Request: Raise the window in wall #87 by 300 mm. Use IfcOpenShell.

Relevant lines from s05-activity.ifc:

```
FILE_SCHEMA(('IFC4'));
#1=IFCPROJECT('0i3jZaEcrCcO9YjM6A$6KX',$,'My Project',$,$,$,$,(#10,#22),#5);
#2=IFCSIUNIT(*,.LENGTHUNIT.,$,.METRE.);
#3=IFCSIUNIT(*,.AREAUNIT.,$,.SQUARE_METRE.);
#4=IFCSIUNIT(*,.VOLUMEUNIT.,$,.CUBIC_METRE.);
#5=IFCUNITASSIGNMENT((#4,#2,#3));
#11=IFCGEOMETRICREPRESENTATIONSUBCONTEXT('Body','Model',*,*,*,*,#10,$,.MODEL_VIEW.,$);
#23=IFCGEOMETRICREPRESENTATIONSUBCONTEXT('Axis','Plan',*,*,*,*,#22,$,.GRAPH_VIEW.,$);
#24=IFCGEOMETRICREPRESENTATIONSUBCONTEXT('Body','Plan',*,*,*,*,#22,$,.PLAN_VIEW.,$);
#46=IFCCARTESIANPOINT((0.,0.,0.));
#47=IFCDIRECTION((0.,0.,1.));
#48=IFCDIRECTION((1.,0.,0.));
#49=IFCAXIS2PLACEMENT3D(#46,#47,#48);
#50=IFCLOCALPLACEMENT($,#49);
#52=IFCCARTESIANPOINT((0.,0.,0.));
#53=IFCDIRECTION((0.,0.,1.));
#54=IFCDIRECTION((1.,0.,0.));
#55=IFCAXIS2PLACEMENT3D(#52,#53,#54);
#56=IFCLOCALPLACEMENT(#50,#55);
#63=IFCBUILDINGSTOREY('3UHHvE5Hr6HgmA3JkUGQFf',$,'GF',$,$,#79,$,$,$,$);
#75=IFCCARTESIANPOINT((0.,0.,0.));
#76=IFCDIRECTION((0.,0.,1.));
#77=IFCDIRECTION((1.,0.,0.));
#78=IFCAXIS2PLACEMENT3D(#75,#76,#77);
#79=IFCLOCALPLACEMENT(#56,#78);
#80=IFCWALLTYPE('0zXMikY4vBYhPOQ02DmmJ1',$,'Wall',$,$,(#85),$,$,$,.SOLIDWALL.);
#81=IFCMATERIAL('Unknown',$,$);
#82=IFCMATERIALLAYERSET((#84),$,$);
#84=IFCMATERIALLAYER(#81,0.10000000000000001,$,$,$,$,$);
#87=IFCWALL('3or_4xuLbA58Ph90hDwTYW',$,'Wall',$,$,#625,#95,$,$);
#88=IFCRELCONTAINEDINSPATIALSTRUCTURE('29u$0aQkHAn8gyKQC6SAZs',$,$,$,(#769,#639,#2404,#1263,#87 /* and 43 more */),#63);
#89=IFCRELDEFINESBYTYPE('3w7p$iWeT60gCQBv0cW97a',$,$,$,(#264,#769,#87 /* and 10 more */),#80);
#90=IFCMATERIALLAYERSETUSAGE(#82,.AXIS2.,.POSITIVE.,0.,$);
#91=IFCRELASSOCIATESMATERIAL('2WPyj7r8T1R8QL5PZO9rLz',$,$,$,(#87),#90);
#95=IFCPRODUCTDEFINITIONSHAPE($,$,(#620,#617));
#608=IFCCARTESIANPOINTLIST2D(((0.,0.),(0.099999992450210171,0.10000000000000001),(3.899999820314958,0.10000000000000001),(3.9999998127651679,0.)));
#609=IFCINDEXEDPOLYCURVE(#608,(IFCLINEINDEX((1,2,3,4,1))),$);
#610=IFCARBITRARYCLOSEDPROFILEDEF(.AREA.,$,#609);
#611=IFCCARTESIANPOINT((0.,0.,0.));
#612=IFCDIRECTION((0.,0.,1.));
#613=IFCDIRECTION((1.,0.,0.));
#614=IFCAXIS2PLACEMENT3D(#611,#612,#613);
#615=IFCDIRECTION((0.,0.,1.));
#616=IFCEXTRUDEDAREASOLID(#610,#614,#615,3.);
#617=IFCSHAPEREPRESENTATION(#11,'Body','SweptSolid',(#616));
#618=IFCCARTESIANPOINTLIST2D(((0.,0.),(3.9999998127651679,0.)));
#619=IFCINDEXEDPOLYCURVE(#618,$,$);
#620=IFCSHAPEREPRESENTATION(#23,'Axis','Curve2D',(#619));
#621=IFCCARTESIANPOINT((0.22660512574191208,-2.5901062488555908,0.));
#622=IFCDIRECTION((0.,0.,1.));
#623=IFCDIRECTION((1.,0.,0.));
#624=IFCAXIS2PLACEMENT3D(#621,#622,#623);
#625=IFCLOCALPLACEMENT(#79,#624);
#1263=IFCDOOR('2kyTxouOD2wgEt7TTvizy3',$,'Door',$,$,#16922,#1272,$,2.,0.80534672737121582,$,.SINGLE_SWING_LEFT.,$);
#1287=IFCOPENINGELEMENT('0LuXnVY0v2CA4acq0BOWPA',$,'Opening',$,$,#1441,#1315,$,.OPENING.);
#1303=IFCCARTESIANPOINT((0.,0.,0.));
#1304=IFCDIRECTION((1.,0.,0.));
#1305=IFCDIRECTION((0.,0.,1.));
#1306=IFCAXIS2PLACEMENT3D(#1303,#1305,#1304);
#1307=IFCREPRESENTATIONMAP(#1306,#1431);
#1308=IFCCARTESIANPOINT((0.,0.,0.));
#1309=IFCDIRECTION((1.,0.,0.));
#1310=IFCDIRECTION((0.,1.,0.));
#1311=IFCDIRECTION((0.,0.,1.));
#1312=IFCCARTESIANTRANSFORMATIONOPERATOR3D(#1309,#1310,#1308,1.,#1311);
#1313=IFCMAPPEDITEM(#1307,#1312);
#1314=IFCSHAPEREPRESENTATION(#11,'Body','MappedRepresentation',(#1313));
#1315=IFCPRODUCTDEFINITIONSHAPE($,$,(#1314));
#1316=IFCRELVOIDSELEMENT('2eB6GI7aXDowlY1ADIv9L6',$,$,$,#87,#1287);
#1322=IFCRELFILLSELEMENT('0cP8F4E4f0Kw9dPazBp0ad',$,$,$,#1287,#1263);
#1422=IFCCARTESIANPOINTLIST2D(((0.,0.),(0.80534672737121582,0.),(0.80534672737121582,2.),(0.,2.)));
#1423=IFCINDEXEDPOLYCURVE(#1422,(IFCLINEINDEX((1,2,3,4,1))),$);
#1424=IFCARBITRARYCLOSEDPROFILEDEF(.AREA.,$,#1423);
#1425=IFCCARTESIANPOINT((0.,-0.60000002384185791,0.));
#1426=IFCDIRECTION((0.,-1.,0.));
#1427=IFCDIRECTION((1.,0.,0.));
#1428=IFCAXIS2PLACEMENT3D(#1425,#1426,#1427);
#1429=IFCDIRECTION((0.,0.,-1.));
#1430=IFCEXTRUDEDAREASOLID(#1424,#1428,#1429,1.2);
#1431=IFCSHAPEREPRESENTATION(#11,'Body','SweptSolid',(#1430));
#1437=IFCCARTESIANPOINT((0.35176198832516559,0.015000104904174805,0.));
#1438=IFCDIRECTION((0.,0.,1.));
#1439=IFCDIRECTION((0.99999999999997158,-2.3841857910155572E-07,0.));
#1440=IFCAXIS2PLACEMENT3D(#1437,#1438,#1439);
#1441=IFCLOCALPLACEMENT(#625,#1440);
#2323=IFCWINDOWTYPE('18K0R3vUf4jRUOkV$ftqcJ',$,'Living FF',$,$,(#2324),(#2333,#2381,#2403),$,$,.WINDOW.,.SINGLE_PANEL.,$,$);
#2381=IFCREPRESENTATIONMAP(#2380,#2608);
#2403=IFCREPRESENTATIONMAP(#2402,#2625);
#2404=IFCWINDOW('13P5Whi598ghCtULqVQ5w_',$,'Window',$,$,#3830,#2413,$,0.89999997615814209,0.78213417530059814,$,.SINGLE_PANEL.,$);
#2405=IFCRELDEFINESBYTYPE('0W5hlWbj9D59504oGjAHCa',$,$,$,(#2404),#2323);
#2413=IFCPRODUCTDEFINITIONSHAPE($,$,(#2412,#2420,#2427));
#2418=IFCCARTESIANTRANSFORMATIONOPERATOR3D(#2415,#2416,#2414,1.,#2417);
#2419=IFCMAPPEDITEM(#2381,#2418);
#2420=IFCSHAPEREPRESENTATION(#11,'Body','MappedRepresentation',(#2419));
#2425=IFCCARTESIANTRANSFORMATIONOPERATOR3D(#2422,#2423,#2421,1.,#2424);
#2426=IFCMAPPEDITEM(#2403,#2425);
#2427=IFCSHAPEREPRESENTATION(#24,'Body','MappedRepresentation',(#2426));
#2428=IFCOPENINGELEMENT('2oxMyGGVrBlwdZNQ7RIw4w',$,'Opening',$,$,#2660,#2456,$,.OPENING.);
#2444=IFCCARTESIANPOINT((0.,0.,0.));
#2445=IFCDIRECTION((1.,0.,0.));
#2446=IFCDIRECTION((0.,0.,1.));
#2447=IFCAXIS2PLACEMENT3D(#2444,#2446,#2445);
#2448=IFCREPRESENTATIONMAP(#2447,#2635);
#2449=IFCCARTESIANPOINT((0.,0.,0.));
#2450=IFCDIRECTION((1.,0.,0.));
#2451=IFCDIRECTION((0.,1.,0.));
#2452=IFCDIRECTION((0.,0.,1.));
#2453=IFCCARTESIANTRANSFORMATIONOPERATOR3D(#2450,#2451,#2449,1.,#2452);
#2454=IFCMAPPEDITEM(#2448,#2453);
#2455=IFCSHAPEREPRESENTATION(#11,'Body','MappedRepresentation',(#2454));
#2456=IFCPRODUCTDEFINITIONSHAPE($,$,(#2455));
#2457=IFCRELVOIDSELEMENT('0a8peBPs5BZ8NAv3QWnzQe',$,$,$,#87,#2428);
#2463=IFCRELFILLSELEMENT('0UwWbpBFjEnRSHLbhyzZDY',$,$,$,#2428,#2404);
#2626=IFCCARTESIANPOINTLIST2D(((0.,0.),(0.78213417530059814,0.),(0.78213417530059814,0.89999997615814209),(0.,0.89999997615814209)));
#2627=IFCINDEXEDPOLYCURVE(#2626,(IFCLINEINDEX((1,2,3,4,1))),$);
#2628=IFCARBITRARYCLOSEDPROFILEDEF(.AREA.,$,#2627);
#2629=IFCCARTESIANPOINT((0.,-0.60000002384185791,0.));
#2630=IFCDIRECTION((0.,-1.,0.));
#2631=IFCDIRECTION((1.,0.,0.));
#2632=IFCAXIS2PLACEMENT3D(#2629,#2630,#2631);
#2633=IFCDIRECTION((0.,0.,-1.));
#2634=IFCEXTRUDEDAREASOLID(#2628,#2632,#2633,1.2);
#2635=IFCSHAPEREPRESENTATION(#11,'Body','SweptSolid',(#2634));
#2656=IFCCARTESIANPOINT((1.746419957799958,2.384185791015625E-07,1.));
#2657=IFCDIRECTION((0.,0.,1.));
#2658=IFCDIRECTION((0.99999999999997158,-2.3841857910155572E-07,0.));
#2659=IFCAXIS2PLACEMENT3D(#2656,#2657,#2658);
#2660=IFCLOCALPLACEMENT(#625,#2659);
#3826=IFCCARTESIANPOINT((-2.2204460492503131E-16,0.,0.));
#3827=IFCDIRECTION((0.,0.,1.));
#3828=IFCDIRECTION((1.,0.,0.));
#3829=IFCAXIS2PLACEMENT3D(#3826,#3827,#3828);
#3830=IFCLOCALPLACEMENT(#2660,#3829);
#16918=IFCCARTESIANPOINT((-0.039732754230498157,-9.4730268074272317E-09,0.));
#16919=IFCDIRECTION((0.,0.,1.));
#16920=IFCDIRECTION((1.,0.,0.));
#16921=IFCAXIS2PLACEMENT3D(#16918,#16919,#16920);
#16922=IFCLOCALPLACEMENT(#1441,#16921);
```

```python
import numpy as np
import ifcopenshell
import ifcopenshell.api.geometry
import ifcopenshell.util.placement
import ifcopenshell.util.unit

model = ifcopenshell.open("s05-activity.ifc")
unit_scale = ifcopenshell.util.unit.calculate_unit_scale(model)

window = model.by_guid("13P5Whi598ghCtULqVQ5w_")
opening = window.FillsVoids[0].RelatingOpeningElement
dz = 0.3 / unit_scale

shift = np.array([0.0, 0.0, dz])
# The window is placed relative to its opening, so it follows when the opening moves.
matrix = ifcopenshell.util.placement.get_local_placement(opening.ObjectPlacement)
matrix[:3, 3] += shift
ifcopenshell.api.geometry.edit_object_placement(
    model, product=opening, matrix=matrix, is_si=False, should_transform_children=True
)

print(f"moved by {dz * unit_scale:+.3f} m")

model.write("s05-activity_v2.ifc")
```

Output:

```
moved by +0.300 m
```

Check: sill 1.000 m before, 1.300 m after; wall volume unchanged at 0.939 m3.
